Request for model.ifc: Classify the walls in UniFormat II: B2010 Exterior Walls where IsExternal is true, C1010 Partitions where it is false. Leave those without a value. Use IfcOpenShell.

First a look at what the model holds.

```python
import ifcopenshell
import ifcopenshell.util.element

model = ifcopenshell.open("model.ifc")
print(model.schema)
print("classifications:", [c.Name for c in model.by_type("IfcClassification")])
values = [ifcopenshell.util.element.get_pset(e, "Pset_WallCommon", "IsExternal") for e in model.by_type("IfcWall")]
for value in (True, False, None):
    print("IsExternal", value, values.count(value))
```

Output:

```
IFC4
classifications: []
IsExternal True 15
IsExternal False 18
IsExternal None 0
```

```python
import ifcopenshell
import ifcopenshell.api.classification
import ifcopenshell.util.element

model = ifcopenshell.open("model.ifc")

system = ifcopenshell.api.classification.add_classification(model, classification="UniFormat II")

walls = model.by_type("IfcWall")
external = {e: ifcopenshell.util.element.get_pset(e, "Pset_WallCommon", "IsExternal") for e in walls}
for flag, code, name in ((True, "B2010", "Exterior Walls"), (False, "C1010", "Partitions")):
    products = [e for e in walls if external[e] is flag]
    ifcopenshell.api.classification.add_reference(
        model, products=products, classification=system, identification=code, name=name
    )
    print(code, len(products))

model.write("model_edited.ifc")
```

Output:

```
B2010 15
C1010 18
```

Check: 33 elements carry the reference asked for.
